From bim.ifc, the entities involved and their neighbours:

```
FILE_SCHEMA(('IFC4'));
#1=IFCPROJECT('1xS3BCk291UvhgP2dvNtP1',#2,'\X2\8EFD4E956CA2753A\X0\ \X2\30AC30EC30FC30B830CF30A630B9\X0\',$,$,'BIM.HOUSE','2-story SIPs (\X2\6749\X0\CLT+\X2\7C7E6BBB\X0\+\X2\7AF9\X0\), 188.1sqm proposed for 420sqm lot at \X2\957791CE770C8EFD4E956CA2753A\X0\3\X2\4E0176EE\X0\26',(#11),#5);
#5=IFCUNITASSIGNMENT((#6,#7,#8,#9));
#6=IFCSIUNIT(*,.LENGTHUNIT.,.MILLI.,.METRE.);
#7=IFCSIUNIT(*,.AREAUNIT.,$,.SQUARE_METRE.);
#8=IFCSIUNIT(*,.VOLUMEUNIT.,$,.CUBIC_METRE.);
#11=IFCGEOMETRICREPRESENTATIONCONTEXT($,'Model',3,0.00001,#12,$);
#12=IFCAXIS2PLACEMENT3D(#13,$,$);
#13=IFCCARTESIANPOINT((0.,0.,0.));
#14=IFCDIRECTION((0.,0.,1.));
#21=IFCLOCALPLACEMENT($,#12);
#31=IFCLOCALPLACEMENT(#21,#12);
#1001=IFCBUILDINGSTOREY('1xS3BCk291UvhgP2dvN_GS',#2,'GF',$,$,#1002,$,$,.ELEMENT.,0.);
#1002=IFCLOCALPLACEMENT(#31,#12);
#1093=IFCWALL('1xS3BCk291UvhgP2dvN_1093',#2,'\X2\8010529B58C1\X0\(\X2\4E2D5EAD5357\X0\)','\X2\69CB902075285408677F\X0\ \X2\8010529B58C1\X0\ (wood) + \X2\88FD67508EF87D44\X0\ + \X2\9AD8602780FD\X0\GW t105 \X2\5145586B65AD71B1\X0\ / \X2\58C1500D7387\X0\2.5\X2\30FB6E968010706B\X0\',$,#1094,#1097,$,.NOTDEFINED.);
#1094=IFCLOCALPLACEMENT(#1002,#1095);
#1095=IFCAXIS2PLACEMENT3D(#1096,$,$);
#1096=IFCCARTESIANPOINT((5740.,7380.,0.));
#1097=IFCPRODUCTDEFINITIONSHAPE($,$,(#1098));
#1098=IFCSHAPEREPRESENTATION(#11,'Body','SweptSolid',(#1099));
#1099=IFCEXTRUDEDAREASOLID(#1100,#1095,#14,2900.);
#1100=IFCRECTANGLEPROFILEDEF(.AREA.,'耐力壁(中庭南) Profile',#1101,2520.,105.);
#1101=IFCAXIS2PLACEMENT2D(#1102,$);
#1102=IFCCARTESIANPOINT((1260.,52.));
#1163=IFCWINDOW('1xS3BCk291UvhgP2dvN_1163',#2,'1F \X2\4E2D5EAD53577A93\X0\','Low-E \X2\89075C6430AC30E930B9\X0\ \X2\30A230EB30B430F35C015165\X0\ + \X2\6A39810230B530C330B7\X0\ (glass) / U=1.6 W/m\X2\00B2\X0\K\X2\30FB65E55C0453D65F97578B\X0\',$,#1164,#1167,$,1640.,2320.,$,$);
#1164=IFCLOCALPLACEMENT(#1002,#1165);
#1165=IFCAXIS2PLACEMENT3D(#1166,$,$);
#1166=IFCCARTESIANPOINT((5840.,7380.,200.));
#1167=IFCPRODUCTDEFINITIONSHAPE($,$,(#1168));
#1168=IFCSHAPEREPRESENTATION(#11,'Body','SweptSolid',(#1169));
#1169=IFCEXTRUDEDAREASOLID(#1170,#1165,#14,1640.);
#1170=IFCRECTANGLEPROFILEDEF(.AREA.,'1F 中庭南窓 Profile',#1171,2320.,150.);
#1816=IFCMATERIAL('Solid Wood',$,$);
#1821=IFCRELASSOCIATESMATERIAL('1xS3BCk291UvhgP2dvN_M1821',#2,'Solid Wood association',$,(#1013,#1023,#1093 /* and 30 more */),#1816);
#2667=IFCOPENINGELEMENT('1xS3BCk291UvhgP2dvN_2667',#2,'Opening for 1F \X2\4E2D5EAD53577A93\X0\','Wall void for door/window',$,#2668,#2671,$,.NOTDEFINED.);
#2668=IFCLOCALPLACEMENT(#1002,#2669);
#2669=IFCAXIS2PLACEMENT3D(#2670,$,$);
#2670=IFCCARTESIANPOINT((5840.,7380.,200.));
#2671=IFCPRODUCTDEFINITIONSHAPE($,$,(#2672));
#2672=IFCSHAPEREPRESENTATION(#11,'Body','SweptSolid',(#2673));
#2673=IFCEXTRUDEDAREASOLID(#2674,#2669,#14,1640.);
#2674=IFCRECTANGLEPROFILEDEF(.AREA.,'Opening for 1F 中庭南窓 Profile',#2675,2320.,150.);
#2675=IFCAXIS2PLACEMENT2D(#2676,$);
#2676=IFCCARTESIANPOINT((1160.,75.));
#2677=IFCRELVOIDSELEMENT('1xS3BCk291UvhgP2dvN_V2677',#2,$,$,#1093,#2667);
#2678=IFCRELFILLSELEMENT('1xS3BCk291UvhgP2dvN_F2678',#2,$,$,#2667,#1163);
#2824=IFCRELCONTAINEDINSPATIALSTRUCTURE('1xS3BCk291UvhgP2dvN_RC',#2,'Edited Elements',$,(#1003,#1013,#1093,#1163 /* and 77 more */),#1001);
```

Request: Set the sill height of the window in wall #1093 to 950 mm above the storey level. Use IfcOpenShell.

```python
import numpy as np
import ifcopenshell
import ifcopenshell.api.geometry
import ifcopenshell.geom
import ifcopenshell.util.element
import ifcopenshell.util.placement
import ifcopenshell.util.shape
import ifcopenshell.util.unit

model = ifcopenshell.open("bim.ifc")
unit_scale = ifcopenshell.util.unit.calculate_unit_scale(model)

window = model.by_guid("1xS3BCk291UvhgP2dvN_1163")
opening = window.FillsVoids[0].RelatingOpeningElement
storey = ifcopenshell.util.element.get_container(window, ifc_class="IfcBuildingStorey")
level = ifcopenshell.util.placement.get_local_placement(storey.ObjectPlacement)[2, 3]

# The opening's origin need not be at the sill, so measure its lowest point.
shape = ifcopenshell.geom.create_shape(ifcopenshell.geom.settings(), opening)
bottom = ifcopenshell.util.shape.get_shape_bottom_elevation(shape, shape.geometry) / unit_scale
dz = level + 950.0 - bottom

shift = np.array([0.0, 0.0, dz])
# The window is not placed relative to its opening, so move both.
for product in (opening, window):
    matrix = ifcopenshell.util.placement.get_local_placement(product.ObjectPlacement)
    matrix[:3, 3] += shift
    ifcopenshell.api.geometry.edit_object_placement(model, product=product, matrix=matrix, is_si=False)

print(f"moved by {dz * unit_scale:+.3f} m")

model.write("bim-out.ifc")
```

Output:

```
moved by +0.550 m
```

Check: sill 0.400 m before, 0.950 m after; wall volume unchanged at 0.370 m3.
